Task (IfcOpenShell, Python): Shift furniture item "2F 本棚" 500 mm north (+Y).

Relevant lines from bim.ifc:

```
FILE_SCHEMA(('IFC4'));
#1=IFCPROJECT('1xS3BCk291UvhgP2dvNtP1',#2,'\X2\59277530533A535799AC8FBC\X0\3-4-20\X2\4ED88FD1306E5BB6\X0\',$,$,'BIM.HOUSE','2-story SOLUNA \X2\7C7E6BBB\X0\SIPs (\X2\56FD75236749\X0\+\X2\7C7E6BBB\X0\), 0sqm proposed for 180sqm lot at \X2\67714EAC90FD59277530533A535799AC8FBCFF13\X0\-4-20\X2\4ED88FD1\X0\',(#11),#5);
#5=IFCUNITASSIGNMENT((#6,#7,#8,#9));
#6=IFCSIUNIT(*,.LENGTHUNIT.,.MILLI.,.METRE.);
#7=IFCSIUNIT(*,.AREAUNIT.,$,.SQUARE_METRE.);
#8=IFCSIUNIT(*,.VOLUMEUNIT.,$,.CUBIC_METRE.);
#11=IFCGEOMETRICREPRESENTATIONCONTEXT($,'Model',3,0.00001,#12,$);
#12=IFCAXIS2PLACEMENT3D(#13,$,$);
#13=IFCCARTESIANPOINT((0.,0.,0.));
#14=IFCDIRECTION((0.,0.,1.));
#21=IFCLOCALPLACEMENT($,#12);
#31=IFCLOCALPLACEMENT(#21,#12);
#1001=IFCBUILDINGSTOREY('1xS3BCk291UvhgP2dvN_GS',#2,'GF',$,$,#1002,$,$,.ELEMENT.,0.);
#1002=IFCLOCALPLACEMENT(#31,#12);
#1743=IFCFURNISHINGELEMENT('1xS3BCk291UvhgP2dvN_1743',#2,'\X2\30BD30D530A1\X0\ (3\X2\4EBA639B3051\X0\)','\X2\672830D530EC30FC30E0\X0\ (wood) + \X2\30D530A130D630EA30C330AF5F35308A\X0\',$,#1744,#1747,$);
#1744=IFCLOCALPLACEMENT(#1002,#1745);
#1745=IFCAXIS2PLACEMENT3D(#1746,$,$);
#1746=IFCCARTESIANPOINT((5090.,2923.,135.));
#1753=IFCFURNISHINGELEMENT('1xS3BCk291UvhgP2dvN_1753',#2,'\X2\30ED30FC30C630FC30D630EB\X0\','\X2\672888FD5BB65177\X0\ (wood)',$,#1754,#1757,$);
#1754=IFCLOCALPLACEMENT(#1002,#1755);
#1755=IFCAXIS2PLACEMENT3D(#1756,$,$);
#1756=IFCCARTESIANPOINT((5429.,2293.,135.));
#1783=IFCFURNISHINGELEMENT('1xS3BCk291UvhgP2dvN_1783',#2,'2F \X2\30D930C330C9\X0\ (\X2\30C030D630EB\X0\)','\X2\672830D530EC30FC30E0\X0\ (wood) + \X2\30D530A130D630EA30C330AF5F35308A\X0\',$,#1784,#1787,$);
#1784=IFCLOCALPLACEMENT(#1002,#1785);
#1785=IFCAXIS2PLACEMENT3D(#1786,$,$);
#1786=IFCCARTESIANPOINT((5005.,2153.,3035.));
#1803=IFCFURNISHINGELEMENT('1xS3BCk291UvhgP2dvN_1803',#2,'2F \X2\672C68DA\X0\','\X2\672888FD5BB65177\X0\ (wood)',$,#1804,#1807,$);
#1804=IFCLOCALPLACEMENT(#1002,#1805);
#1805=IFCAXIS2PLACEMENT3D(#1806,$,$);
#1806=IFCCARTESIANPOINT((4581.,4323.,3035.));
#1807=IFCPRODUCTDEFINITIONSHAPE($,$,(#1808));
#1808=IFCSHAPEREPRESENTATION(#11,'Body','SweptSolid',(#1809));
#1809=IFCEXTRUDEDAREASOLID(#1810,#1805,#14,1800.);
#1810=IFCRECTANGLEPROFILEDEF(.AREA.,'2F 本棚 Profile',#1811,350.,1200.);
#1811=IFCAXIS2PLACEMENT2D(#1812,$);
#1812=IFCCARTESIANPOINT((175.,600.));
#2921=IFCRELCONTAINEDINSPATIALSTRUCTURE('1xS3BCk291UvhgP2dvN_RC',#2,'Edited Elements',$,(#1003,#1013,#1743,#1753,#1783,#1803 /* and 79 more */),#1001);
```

```python
import ifcopenshell
import ifcopenshell.api.geometry
import ifcopenshell.util.placement
import ifcopenshell.util.unit

model = ifcopenshell.open("bim.ifc")
unit_scale = ifcopenshell.util.unit.calculate_unit_scale(model)

item = model.by_guid("1xS3BCk291UvhgP2dvN_1803")
matrix = ifcopenshell.util.placement.get_local_placement(item.ObjectPlacement)
matrix[1, 3] += 0.5 / unit_scale
ifcopenshell.api.geometry.edit_object_placement(model, product=item, matrix=matrix, is_si=False)

print(ifcopenshell.util.placement.get_local_placement(item.ObjectPlacement).round(3) + 0.0)

model.write("bim_v2.ifc")
```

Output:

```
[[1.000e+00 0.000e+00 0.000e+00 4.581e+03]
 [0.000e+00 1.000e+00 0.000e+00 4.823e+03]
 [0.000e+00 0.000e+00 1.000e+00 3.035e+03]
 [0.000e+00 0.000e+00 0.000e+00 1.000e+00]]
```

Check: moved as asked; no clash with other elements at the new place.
